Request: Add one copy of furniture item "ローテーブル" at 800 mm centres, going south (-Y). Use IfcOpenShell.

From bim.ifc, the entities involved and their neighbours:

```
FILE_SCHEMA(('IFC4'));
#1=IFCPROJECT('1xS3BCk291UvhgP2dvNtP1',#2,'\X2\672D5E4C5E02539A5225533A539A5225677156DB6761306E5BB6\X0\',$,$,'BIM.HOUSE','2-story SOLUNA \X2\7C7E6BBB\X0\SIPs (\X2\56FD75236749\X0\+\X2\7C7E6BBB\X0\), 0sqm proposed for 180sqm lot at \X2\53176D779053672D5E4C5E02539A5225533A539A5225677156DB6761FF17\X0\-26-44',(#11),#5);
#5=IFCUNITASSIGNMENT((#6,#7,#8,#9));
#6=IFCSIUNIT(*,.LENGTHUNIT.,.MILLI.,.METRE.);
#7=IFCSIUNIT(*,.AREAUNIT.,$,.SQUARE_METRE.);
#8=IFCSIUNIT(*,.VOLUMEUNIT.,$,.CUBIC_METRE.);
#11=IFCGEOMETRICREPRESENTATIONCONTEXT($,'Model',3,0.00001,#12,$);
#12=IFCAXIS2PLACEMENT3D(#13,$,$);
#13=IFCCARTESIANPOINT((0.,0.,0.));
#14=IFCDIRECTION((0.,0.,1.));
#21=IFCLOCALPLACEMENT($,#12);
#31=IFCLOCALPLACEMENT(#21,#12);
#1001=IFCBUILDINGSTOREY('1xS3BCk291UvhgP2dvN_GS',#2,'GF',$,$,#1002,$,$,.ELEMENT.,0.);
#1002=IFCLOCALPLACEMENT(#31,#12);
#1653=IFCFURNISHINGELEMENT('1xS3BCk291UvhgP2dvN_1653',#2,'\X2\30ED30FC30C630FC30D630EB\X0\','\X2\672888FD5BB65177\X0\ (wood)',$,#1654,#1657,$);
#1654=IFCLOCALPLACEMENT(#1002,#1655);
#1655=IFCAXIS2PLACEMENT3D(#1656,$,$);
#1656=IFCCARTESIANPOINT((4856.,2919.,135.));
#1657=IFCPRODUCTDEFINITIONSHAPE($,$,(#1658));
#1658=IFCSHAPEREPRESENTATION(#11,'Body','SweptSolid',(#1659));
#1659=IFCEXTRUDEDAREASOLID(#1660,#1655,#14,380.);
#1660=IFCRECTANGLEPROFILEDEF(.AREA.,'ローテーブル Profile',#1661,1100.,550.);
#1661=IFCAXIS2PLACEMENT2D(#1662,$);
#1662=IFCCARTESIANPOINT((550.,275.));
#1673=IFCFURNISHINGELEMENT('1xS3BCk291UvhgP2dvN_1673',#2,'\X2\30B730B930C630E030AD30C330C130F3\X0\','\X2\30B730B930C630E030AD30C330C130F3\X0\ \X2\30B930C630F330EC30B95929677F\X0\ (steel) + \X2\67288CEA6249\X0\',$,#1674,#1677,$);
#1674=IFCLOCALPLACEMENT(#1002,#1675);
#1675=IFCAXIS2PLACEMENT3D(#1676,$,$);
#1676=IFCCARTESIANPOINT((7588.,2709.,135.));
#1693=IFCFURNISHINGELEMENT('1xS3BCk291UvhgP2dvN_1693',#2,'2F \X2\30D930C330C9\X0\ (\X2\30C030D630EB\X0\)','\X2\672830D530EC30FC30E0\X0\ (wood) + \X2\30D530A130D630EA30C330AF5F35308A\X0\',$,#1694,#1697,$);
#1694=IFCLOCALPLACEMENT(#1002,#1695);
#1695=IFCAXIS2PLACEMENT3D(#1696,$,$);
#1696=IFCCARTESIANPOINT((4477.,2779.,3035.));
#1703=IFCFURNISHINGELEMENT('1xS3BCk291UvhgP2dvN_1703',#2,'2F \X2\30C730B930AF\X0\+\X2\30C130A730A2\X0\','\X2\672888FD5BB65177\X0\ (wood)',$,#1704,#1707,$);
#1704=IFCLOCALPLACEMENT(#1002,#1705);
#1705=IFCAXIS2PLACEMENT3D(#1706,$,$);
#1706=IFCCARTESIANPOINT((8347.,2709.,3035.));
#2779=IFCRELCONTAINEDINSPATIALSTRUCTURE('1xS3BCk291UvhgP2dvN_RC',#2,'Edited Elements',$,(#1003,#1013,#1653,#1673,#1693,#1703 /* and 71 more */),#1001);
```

```python
import numpy as np
import ifcopenshell
import ifcopenshell.api.geometry
import ifcopenshell.api.root
import ifcopenshell.util.element
import ifcopenshell.util.placement
import ifcopenshell.util.unit

model = ifcopenshell.open("bim.ifc")
unit_scale = ifcopenshell.util.unit.calculate_unit_scale(model)


def reuse_history(source, copy):
    """copy_class also copies each property set's owner history, people and application; keep the originals."""
    for rel in copy.IsDefinedBy:
        if rel.is_a("IfcRelDefinesByProperties") and (history := rel.RelatingPropertyDefinition.OwnerHistory):
            rel.RelatingPropertyDefinition.OwnerHistory = source.OwnerHistory
            ifcopenshell.util.element.remove_deep2(model, history)


source = model.by_id(1653)
base = ifcopenshell.util.placement.get_local_placement(source.ObjectPlacement)
step = np.array([0.0, -1.0, 0.0]) * 0.8 / unit_scale

for i in range(1, 2):
    copy = ifcopenshell.api.root.copy_class(model, product=source)
    copy.Representation = ifcopenshell.util.element.copy_deep(
        model, source.Representation, exclude=["IfcGeometricRepresentationContext", "IfcRepresentationMap"]
    )
    reuse_history(source, copy)
    matrix = base.copy()
    matrix[:3, 3] += i * step
    print("added at", matrix[:3, 3].round(3) + 0.0)
    ifcopenshell.api.geometry.edit_object_placement(model, product=copy, matrix=matrix, is_si=False)

model.write("bim_v2.ifc")
```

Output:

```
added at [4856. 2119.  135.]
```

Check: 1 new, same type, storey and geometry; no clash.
